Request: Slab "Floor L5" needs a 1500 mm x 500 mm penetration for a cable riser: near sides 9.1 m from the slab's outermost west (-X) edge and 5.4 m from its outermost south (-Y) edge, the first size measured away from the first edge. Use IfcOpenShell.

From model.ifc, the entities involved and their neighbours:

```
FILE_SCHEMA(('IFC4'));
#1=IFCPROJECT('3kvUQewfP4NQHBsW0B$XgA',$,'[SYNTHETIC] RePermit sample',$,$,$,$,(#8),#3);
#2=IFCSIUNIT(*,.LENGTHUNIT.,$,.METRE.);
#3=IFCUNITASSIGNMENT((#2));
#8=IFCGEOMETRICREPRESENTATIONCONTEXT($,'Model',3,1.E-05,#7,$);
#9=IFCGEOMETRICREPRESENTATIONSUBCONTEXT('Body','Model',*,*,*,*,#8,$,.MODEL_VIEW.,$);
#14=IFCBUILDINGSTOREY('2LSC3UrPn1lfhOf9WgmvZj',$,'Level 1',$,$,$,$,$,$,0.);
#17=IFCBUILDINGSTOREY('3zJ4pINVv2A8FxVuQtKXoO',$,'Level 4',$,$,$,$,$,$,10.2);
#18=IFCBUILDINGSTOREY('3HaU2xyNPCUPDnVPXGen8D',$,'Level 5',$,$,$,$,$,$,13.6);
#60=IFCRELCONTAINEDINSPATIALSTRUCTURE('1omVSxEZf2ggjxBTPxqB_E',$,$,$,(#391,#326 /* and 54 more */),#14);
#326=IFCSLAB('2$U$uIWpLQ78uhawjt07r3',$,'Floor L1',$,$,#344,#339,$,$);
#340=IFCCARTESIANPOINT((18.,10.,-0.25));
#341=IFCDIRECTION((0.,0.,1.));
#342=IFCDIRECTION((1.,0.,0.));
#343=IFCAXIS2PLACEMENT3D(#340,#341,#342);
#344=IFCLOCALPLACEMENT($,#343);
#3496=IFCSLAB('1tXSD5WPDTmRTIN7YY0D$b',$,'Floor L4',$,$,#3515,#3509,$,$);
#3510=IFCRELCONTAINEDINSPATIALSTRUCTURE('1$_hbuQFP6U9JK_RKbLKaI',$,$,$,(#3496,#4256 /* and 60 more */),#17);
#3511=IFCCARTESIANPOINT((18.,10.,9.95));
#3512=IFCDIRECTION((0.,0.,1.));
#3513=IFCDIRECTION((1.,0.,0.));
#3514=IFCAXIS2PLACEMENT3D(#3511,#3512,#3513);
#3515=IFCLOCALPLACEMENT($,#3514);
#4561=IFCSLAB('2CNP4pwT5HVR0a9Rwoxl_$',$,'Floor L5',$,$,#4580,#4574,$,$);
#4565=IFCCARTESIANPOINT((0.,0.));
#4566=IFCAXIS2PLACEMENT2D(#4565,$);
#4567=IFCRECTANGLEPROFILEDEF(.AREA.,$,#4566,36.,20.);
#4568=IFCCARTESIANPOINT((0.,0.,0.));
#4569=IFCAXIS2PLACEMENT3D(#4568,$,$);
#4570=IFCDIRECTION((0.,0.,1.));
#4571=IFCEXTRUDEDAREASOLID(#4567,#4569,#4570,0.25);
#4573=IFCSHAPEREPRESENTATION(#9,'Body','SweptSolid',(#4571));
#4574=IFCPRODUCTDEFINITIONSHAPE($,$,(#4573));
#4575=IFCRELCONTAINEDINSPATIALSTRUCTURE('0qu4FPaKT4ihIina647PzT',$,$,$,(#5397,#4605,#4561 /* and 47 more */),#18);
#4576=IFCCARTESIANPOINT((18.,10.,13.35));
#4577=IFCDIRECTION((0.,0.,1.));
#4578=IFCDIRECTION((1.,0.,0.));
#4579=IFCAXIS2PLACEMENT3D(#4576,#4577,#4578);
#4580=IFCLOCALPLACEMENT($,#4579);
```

```python
import numpy as np
import ifcopenshell
import ifcopenshell.api.feature
import ifcopenshell.api.geometry
import ifcopenshell.api.root
import ifcopenshell.geom
import ifcopenshell.util.placement
import ifcopenshell.util.representation
import ifcopenshell.util.shape
import ifcopenshell.util.unit

model = ifcopenshell.open("model.ifc")
unit_scale = ifcopenshell.util.unit.calculate_unit_scale(model)
settings = ifcopenshell.geom.settings()


def volume(element):
    """Net volume in cubic metres, openings subtracted."""
    shape = ifcopenshell.geom.create_shape(settings, element)
    return ifcopenshell.util.shape.get_volume(shape.geometry)


slab = model.by_guid("2CNP4pwT5HVR0a9Rwoxl_$")
before = volume(slab)

# Extent in the slab's own axes, in metres. The edges named are its -X and -Y sides.
slab_shape = ifcopenshell.geom.create_shape(settings, slab)
vertices = ifcopenshell.util.shape.get_vertices(slab_shape.geometry)
x_min, y_min, bottom = vertices.min(axis=0)
top = vertices[:, 2].max()

opening = ifcopenshell.api.root.create_entity(model, ifc_class="IfcOpeningElement", name="Cable riser opening", predefined_type="OPENING")
context = ifcopenshell.util.representation.get_context(model, "Model", "Body", "MODEL_VIEW")
width, depth = 1.5, 0.5
outline = [(0.0, 0.0), (width, 0.0), (width, depth), (0.0, depth), (0.0, 0.0)]
# Overshoot both faces by 50 mm so the cut is clean.
shape = ifcopenshell.api.geometry.add_slab_representation(
    model, context=context, depth=top - bottom + 0.1, polyline=outline
)
ifcopenshell.api.geometry.assign_representation(model, product=opening, representation=shape)

matrix = ifcopenshell.util.placement.get_local_placement(slab.ObjectPlacement)
matrix[:, 3] = matrix @ np.append(np.array([x_min + 9.1, y_min + 5.4, bottom - 0.05]) / unit_scale, 1.0)
ifcopenshell.api.geometry.edit_object_placement(model, product=opening, matrix=matrix, is_si=False)
ifcopenshell.api.feature.add_feature(model, feature=opening, element=slab)

after = volume(slab)

print(f"slab volume {before:.3f} -> {after:.3f} m3")

model.write("model_v2.ifc")
```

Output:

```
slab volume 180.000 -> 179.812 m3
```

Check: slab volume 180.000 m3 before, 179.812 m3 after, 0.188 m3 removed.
